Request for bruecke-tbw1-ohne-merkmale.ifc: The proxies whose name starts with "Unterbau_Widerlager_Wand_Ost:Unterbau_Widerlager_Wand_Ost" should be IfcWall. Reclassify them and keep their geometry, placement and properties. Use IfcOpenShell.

First a look at what the model holds.

```python
import re

import ifcopenshell

model = ifcopenshell.open("bruecke-tbw1-ohne-merkmale.ifc")
print(model.schema)
seen = {}
for e in model.by_type("IfcBuildingElementProxy"):
    name = re.sub(r":\d+(:\d+)?$", "", e.Name or "")  # drop the element id that some exporters append
    seen[name] = seen.get(name, 0) + 1
for name, count in sorted(seen.items()):
    print(count, "x", name)
```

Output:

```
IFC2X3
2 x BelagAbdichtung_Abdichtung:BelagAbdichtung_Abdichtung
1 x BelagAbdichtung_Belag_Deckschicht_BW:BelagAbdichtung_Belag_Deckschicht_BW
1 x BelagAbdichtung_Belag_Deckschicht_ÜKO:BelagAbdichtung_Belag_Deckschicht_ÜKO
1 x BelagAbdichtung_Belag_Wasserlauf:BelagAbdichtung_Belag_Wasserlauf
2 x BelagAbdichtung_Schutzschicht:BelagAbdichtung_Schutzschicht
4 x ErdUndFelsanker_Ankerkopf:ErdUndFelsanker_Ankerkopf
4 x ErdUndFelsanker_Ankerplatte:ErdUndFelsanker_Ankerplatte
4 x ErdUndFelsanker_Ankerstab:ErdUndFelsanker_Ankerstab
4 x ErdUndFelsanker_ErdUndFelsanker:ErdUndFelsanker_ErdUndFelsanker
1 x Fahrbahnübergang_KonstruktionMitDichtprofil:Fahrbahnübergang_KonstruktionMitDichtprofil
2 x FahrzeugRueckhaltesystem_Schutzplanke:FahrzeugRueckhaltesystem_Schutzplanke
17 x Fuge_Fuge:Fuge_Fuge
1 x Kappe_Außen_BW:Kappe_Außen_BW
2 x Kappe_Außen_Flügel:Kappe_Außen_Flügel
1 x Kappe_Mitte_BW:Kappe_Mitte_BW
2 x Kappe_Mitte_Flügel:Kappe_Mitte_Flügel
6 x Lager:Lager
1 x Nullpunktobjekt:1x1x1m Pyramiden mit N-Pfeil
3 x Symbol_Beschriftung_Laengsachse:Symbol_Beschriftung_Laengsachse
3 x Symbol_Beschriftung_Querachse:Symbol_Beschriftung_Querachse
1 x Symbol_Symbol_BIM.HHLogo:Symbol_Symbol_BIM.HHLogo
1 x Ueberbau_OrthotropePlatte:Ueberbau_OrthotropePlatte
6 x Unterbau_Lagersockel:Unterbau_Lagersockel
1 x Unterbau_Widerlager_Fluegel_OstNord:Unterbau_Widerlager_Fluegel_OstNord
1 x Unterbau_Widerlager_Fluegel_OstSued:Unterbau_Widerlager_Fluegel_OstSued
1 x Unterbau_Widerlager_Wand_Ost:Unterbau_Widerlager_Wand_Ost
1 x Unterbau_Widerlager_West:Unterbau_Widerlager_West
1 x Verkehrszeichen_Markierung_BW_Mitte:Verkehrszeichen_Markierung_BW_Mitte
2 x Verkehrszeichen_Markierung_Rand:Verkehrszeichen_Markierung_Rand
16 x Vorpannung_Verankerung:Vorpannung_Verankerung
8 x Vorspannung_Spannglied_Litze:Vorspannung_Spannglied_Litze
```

```python
import ifcopenshell
import ifcopenshell.api.root

model = ifcopenshell.open("bruecke-tbw1-ohne-merkmale.ifc")

proxies = [e.id() for e in model.by_type("IfcBuildingElementProxy") if (e.Name or "").startswith("Unterbau_Widerlager_Wand_Ost:Unterbau_Widerlager_Wand_Ost")]
for step_id in proxies:
    proxy = model.by_id(step_id)
    # Reclassifying a typed element also reclassifies its type and the type's other occurrences.
    if proxy.is_a("IfcBuildingElementProxy"):
        ifcopenshell.api.root.reassign_class(model, product=proxy, ifc_class="IfcWall")

print(sum(model.by_id(i).is_a("IfcWall") for i in proxies), "reclassified")

model.write("bruecke-tbw1-ohne-merkmale_edited.ifc")
```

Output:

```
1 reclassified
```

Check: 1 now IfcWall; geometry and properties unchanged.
